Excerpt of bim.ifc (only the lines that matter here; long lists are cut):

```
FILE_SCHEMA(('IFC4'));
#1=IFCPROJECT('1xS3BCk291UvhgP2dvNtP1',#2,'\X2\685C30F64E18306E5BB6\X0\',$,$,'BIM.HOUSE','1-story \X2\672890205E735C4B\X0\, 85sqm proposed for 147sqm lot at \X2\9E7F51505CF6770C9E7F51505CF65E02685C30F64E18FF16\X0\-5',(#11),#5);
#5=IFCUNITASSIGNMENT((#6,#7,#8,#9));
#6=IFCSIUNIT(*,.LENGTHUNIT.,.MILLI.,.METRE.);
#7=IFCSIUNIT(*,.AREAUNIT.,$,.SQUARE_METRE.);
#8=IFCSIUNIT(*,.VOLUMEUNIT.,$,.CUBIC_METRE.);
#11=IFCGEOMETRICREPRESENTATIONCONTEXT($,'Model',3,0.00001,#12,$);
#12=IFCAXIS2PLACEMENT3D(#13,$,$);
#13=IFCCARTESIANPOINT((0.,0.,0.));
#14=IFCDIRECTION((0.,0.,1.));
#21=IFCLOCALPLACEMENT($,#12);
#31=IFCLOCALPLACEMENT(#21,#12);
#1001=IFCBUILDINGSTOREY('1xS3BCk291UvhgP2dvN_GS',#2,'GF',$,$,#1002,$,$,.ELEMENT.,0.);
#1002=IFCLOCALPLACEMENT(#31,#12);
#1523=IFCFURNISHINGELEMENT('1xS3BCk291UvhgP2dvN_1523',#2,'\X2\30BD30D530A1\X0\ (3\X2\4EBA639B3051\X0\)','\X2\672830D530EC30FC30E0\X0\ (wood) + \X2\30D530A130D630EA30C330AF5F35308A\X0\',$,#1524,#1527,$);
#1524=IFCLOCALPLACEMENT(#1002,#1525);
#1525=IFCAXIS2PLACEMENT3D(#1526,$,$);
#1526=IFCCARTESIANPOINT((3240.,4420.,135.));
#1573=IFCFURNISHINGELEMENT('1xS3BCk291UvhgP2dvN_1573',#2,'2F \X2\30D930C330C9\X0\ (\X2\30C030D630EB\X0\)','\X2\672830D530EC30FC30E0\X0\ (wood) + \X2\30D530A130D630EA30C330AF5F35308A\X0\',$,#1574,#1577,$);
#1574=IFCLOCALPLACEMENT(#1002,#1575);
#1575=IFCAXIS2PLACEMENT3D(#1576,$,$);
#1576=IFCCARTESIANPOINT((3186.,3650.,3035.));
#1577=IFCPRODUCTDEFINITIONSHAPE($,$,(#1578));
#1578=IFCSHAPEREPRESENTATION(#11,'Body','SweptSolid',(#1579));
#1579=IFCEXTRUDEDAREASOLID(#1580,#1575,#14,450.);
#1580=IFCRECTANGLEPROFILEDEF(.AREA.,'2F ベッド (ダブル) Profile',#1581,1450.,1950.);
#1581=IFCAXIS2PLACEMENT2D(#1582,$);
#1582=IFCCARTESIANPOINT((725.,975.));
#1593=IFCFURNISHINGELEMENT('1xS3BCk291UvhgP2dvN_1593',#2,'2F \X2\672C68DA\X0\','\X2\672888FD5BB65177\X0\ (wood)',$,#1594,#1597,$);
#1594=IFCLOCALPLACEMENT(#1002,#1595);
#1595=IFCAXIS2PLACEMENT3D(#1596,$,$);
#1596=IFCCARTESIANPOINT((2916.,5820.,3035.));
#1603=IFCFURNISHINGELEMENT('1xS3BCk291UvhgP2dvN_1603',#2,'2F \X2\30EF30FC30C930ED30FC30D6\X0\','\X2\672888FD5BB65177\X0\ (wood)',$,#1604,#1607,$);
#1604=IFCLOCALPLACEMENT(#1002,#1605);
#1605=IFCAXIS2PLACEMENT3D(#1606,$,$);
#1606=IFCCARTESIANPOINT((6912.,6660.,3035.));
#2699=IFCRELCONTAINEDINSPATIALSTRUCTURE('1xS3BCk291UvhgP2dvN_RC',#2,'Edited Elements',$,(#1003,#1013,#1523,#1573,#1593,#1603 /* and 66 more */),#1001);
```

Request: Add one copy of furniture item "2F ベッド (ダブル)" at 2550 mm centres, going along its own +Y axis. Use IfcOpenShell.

```python
import ifcopenshell
import ifcopenshell.api.geometry
import ifcopenshell.api.root
import ifcopenshell.util.element
import ifcopenshell.util.placement

model = ifcopenshell.open("bim.ifc")


def reuse_history(source, copy):
    """copy_class also copies each property set's owner history, people and application; keep the originals."""
    for rel in copy.IsDefinedBy:
        if rel.is_a("IfcRelDefinesByProperties") and (history := rel.RelatingPropertyDefinition.OwnerHistory):
            rel.RelatingPropertyDefinition.OwnerHistory = source.OwnerHistory
            ifcopenshell.util.element.remove_deep2(model, history)


source = model.by_guid("1xS3BCk291UvhgP2dvN_1573")
base = ifcopenshell.util.placement.get_local_placement(source.ObjectPlacement)
step = base[:3, 1] * 2550.0

for i in range(1, 2):
    copy = ifcopenshell.api.root.copy_class(model, product=source)
    copy.Representation = ifcopenshell.util.element.copy_deep(
        model, source.Representation, exclude=["IfcGeometricRepresentationContext", "IfcRepresentationMap"]
    )
    reuse_history(source, copy)
    matrix = base.copy()
    matrix[:3, 3] += i * step
    print("added at", matrix[:3, 3].round(3) + 0.0)
    ifcopenshell.api.geometry.edit_object_placement(model, product=copy, matrix=matrix, is_si=False)

model.write("bim_v2.ifc")
```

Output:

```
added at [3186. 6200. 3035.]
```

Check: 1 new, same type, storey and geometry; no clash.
